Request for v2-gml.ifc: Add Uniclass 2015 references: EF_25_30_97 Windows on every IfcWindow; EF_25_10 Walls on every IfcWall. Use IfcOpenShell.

First a look at what the model holds.

```python
import ifcopenshell

model = ifcopenshell.open("v2-gml.ifc")
print(model.schema)
print("classifications:", [c.Name for c in model.by_type("IfcClassification")])
for ifc_class in ("IfcDoor", "IfcRoof", "IfcStair", "IfcWall", "IfcWindow"):
    print(ifc_class, len(model.by_type(ifc_class)))
```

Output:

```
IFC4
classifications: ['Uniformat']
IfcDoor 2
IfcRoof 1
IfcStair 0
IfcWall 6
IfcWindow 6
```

```python
import ifcopenshell
import ifcopenshell.api.classification

model = ifcopenshell.open("v2-gml.ifc")

system = ifcopenshell.api.classification.add_classification(model, classification="Uniclass 2015")

codes = {
    "IfcWindow": ("EF_25_30_97", "Windows"),
    "IfcWall": ("EF_25_10", "Walls"),
}
for ifc_class, (code, name) in codes.items():
    products = model.by_type(ifc_class)
    ifcopenshell.api.classification.add_reference(
        model, products=products, classification=system, identification=code, name=name
    )
    print(code, len(products))

model.write("v2-gml_v2.ifc")
```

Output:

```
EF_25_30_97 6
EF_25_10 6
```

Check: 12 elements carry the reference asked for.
